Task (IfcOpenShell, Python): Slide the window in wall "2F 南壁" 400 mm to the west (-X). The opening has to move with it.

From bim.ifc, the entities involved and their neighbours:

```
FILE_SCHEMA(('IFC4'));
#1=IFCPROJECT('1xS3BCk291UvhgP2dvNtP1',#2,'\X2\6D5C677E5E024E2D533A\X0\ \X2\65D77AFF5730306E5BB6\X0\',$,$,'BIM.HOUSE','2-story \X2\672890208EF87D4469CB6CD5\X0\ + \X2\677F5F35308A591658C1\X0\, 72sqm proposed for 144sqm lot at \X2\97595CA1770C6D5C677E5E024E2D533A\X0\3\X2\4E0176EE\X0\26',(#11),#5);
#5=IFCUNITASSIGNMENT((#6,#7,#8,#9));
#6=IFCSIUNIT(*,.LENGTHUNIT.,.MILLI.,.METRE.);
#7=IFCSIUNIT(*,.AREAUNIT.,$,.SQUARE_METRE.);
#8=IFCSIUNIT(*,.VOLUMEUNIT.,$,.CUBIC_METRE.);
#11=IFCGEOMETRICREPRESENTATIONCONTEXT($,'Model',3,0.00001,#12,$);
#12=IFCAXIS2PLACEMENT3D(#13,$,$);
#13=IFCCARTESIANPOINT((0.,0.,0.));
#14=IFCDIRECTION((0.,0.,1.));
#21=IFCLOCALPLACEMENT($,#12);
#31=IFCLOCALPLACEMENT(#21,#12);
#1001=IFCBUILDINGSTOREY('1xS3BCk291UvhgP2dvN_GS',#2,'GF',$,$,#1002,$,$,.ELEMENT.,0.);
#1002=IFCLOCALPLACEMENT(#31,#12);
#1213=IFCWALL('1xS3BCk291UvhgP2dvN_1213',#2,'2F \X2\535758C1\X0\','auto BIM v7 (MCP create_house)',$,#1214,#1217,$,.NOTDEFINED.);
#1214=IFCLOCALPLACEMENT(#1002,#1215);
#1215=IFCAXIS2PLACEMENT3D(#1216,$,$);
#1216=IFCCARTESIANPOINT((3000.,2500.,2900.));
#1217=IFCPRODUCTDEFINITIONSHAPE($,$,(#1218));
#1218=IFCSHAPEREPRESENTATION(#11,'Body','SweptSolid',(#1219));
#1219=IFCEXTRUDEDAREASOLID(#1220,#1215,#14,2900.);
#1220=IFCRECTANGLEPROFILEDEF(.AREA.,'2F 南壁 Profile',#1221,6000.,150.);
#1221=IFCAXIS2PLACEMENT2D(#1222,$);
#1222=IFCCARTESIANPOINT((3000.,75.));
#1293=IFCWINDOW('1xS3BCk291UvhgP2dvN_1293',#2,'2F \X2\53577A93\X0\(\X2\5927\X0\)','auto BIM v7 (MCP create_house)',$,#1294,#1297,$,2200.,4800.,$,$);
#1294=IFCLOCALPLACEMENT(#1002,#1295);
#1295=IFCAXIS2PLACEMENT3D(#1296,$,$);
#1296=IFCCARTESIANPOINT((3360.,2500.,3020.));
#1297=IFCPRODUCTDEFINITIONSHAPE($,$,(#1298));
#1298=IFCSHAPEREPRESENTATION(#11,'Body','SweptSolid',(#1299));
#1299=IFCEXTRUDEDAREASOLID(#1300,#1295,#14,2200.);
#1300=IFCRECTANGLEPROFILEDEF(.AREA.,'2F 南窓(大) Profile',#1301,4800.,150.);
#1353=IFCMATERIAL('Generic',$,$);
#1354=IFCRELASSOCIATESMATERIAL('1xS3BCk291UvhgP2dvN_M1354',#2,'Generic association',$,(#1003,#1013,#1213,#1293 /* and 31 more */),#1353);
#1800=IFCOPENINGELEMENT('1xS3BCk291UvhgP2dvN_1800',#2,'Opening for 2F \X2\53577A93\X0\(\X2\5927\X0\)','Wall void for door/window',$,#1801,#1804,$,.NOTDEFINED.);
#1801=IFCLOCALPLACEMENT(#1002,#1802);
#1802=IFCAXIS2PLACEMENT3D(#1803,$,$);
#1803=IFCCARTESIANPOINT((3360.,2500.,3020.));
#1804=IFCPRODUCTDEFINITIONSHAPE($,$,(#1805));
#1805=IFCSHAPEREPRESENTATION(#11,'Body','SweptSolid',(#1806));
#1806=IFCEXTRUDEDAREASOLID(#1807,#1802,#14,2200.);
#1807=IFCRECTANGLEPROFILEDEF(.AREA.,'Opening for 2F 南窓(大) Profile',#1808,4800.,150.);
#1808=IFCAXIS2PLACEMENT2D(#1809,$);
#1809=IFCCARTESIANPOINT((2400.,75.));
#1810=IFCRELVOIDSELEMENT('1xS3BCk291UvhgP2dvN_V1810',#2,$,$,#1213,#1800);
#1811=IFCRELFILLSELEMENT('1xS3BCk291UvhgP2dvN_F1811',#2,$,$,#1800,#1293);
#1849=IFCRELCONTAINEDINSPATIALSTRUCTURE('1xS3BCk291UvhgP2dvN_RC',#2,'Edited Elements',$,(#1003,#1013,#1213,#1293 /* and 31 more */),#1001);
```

```python
import ifcopenshell
import ifcopenshell.api.geometry
import ifcopenshell.util.placement

model = ifcopenshell.open("bim.ifc")

window = model.by_guid("1xS3BCk291UvhgP2dvN_1293")
opening = window.FillsVoids[0].RelatingOpeningElement
wall = opening.VoidsElements[0].RelatingBuildingElement

wall_matrix = ifcopenshell.util.placement.get_local_placement(wall.ObjectPlacement)
shift = wall_matrix[:3, 0] * -400.0
before = ifcopenshell.util.placement.get_local_placement(window.ObjectPlacement)[:3, 3].copy()

# The window is not placed relative to its opening, so move both.
for product in (opening, window):
    matrix = ifcopenshell.util.placement.get_local_placement(product.ObjectPlacement)
    matrix[:3, 3] += shift
    ifcopenshell.api.geometry.edit_object_placement(model, product=product, matrix=matrix, is_si=False)

after = ifcopenshell.util.placement.get_local_placement(window.ObjectPlacement)[:3, 3]
print("window moved by", (after - before).round(3) + 0.0)

model.write("bim_rev.ifc")
```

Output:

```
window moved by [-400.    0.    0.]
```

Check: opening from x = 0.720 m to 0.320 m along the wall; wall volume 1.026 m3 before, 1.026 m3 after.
